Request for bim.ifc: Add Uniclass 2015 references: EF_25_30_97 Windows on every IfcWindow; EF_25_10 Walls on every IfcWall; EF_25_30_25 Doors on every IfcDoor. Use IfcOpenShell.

First a look at what the model holds.

```python
import ifcopenshell

model = ifcopenshell.open("bim.ifc")
print(model.schema)
print("classifications:", [c.Name for c in model.by_type("IfcClassification")])
for ifc_class in ("IfcDoor", "IfcRoof", "IfcStair", "IfcWall", "IfcWindow"):
    print(ifc_class, len(model.by_type(ifc_class)))
```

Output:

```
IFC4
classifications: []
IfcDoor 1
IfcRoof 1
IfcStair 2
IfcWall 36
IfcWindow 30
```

```python
import ifcopenshell
import ifcopenshell.api.classification

model = ifcopenshell.open("bim.ifc")

system = ifcopenshell.api.classification.add_classification(model, classification="Uniclass 2015")

codes = {
    "IfcWindow": ("EF_25_30_97", "Windows"),
    "IfcWall": ("EF_25_10", "Walls"),
    "IfcDoor": ("EF_25_30_25", "Doors"),
}
for ifc_class, (code, name) in codes.items():
    products = model.by_type(ifc_class)
    ifcopenshell.api.classification.add_reference(
        model, products=products, classification=system, identification=code, name=name
    )
    print(code, len(products))

model.write("bim-out.ifc")
```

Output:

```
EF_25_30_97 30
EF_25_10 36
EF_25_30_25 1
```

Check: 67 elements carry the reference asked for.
